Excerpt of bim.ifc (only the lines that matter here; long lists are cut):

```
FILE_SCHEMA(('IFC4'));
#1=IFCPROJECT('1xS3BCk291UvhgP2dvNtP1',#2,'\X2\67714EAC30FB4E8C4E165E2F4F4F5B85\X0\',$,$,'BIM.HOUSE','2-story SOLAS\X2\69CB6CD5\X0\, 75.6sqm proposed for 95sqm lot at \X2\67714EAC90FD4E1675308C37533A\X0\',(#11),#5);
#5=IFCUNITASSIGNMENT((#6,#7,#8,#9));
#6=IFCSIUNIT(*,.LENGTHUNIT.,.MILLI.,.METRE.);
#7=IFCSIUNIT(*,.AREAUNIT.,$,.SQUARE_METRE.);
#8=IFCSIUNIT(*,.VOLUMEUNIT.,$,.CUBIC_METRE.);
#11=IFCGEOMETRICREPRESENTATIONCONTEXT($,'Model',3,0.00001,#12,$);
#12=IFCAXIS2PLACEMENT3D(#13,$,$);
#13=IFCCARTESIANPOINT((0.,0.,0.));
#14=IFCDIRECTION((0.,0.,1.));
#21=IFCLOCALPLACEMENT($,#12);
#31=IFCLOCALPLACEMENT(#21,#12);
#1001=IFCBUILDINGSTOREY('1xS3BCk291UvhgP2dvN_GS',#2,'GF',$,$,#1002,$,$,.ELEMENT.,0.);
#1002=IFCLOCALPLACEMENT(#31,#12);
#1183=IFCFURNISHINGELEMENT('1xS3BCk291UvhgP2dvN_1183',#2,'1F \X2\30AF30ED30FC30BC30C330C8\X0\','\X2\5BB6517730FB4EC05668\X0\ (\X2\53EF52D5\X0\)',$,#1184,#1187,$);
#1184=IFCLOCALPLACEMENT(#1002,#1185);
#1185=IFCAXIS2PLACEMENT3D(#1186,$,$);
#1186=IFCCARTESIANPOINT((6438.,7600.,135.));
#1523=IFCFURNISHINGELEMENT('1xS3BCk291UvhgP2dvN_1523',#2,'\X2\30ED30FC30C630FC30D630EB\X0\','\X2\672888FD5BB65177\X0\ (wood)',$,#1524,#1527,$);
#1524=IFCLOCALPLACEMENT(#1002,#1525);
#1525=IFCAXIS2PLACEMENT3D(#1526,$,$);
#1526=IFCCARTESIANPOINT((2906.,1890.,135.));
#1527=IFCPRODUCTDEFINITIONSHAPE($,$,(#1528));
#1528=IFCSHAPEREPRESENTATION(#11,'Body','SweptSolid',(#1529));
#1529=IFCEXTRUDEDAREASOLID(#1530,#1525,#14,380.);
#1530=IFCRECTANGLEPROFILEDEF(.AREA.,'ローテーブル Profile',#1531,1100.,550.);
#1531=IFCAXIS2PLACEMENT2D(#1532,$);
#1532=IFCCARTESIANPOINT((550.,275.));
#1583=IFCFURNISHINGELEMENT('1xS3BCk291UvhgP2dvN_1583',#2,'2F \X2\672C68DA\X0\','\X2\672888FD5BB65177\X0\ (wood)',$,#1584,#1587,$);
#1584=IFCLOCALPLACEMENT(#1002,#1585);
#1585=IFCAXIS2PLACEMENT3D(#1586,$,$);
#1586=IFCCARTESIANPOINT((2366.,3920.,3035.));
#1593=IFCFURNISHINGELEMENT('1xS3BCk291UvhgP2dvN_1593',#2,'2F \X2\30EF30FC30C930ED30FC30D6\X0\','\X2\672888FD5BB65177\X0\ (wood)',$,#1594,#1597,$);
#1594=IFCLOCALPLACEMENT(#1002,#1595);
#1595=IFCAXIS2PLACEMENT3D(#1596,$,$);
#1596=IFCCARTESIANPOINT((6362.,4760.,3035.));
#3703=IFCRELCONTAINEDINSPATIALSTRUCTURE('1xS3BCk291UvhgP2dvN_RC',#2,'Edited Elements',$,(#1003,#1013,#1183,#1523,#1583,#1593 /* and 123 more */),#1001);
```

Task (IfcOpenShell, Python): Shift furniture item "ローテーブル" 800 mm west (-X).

```python
import ifcopenshell
import ifcopenshell.api.geometry
import ifcopenshell.util.placement
import ifcopenshell.util.unit

model = ifcopenshell.open("bim.ifc")
unit_scale = ifcopenshell.util.unit.calculate_unit_scale(model)

item = model.by_guid("1xS3BCk291UvhgP2dvN_1523")
matrix = ifcopenshell.util.placement.get_local_placement(item.ObjectPlacement)
matrix[0, 3] -= 0.8 / unit_scale
ifcopenshell.api.geometry.edit_object_placement(model, product=item, matrix=matrix, is_si=False)

print(ifcopenshell.util.placement.get_local_placement(item.ObjectPlacement).round(3) + 0.0)

model.write("bim-out.ifc")
```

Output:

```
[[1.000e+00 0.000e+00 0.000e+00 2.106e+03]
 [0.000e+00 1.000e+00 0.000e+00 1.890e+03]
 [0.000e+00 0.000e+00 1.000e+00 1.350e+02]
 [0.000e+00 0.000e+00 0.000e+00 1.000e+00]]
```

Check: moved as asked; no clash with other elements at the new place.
